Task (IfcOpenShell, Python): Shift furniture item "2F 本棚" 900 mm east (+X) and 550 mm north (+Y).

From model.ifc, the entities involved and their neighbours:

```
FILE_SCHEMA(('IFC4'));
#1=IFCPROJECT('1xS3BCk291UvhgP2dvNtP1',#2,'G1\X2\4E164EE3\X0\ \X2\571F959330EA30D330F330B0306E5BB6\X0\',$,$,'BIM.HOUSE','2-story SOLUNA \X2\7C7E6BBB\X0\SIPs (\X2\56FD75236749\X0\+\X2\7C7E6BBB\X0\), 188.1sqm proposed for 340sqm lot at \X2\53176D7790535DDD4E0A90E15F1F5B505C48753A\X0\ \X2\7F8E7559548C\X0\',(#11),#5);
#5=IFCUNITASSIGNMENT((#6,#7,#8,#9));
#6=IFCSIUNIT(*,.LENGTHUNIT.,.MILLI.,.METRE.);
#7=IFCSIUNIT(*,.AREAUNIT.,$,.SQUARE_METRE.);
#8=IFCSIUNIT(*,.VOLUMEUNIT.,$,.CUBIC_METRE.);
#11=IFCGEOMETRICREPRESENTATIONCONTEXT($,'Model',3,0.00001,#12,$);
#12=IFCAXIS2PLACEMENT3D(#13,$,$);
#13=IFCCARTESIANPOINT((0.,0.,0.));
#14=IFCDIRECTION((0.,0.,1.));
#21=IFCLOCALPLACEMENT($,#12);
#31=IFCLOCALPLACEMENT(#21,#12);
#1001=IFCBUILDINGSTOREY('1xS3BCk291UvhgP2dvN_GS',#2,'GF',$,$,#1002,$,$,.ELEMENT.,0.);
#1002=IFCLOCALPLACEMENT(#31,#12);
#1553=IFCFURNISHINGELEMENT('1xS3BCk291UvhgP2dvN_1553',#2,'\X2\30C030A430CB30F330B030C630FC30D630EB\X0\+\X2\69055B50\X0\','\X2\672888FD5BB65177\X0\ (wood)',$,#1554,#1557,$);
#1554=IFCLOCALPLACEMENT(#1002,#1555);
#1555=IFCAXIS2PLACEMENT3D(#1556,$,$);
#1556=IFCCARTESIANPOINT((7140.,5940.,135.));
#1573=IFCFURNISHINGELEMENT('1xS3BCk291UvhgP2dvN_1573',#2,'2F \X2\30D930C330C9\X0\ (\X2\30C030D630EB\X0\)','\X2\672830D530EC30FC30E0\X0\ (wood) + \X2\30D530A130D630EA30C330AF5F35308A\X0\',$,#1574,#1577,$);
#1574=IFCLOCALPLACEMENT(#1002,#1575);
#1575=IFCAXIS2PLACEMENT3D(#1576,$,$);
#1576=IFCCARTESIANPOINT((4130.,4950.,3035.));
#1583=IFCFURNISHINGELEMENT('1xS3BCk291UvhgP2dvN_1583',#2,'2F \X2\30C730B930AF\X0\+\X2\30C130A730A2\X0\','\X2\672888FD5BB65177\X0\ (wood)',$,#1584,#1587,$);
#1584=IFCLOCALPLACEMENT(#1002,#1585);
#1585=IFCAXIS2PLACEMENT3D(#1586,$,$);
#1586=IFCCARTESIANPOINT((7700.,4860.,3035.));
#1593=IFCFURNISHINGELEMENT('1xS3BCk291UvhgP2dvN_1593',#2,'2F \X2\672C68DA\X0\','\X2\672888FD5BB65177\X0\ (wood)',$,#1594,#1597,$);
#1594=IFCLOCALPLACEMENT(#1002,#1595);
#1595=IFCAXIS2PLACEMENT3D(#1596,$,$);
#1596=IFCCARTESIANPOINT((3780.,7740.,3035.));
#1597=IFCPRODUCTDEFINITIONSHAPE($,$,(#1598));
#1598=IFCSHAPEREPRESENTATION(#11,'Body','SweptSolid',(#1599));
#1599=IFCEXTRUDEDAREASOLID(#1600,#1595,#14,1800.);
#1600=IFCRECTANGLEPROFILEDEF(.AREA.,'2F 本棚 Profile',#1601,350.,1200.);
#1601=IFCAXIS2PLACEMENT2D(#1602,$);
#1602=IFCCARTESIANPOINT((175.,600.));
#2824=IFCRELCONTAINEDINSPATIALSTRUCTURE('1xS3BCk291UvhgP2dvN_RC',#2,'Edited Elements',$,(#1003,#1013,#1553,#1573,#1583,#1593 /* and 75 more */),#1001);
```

```python
import ifcopenshell
import ifcopenshell.api.geometry
import ifcopenshell.util.placement
import ifcopenshell.util.unit

model = ifcopenshell.open("model.ifc")
unit_scale = ifcopenshell.util.unit.calculate_unit_scale(model)

item = model.by_guid("1xS3BCk291UvhgP2dvN_1593")
matrix = ifcopenshell.util.placement.get_local_placement(item.ObjectPlacement)
matrix[0, 3] += 0.9 / unit_scale
matrix[1, 3] += 0.55 / unit_scale
ifcopenshell.api.geometry.edit_object_placement(model, product=item, matrix=matrix, is_si=False)

print(ifcopenshell.util.placement.get_local_placement(item.ObjectPlacement).round(3) + 0.0)

model.write("model_rev.ifc")
```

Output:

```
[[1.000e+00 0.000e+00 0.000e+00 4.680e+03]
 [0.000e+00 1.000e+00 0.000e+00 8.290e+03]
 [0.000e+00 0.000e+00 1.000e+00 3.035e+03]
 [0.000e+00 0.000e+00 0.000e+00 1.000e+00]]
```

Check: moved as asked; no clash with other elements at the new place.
